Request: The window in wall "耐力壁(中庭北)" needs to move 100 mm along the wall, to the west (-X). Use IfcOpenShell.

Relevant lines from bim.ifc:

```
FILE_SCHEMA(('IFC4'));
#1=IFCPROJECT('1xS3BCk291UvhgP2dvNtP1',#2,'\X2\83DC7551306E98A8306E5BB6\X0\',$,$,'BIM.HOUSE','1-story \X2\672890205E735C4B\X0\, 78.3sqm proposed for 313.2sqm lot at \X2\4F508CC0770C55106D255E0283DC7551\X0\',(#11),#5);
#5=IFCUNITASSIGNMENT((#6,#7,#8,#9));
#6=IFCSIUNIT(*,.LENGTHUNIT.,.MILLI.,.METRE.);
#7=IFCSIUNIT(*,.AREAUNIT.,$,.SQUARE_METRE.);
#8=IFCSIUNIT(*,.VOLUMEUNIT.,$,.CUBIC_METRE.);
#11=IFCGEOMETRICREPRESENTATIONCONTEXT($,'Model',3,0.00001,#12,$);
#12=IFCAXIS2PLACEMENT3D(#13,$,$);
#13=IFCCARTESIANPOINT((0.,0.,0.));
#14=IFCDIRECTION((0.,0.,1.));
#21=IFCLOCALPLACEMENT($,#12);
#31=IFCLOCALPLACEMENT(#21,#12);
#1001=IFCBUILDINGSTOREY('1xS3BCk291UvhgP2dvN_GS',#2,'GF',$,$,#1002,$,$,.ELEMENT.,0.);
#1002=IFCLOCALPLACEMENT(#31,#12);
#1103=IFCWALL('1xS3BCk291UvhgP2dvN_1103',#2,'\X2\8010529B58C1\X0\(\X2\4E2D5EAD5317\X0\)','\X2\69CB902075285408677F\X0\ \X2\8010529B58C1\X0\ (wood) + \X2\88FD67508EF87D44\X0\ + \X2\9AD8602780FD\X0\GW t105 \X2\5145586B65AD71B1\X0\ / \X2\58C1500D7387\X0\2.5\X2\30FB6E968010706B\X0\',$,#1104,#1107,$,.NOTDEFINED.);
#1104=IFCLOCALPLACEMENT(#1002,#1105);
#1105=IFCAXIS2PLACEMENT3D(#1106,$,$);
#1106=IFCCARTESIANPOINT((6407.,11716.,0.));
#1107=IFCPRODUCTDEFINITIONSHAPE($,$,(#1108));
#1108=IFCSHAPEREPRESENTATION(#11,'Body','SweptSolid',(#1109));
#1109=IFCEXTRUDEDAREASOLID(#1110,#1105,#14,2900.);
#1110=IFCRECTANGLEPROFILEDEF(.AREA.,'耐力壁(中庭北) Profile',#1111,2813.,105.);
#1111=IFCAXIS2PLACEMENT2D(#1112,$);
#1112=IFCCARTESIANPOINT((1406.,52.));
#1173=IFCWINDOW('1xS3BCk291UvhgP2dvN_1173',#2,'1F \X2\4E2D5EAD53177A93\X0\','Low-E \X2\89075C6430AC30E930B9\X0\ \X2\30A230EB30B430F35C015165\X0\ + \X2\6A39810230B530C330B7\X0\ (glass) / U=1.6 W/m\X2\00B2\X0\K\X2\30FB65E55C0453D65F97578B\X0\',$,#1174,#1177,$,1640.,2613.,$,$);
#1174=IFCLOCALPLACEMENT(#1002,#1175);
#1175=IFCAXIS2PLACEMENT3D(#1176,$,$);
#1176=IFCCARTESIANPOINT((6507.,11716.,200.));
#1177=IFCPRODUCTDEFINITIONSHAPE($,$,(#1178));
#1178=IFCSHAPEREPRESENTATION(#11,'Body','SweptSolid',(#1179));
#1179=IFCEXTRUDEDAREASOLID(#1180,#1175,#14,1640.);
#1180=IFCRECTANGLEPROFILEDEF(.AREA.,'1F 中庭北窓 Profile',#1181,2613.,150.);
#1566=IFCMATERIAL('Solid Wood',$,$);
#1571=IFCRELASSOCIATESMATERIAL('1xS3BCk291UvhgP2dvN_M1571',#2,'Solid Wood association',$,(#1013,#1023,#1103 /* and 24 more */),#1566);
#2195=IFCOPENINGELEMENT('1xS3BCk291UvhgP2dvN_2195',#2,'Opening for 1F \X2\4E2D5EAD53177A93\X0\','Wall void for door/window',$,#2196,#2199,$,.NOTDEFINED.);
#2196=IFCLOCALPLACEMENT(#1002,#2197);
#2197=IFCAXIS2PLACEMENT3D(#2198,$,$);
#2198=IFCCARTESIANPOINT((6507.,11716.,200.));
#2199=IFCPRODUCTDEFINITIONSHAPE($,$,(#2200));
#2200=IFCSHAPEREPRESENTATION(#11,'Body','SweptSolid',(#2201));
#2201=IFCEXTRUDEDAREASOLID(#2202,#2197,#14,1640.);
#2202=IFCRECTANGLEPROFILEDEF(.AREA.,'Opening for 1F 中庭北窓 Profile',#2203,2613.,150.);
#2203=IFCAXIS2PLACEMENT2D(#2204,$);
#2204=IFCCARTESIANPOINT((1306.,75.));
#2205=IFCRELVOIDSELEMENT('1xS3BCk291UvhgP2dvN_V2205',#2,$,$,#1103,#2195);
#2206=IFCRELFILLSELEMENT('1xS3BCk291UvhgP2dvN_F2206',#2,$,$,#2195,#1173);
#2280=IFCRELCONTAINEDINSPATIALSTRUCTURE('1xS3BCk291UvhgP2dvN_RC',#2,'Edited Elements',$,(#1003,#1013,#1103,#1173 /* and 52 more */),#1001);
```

```python
import ifcopenshell
import ifcopenshell.api.geometry
import ifcopenshell.util.placement
import ifcopenshell.util.unit

model = ifcopenshell.open("bim.ifc")
unit_scale = ifcopenshell.util.unit.calculate_unit_scale(model)

window = model.by_guid("1xS3BCk291UvhgP2dvN_1173")
opening = window.FillsVoids[0].RelatingOpeningElement
wall = opening.VoidsElements[0].RelatingBuildingElement

wall_matrix = ifcopenshell.util.placement.get_local_placement(wall.ObjectPlacement)
shift = wall_matrix[:3, 0] * -0.1 / unit_scale
before = ifcopenshell.util.placement.get_local_placement(window.ObjectPlacement)[:3, 3].copy()

# The window is not placed relative to its opening, so move both.
for product in (opening, window):
    matrix = ifcopenshell.util.placement.get_local_placement(product.ObjectPlacement)
    matrix[:3, 3] += shift
    ifcopenshell.api.geometry.edit_object_placement(model, product=product, matrix=matrix, is_si=False)

after = ifcopenshell.util.placement.get_local_placement(window.ObjectPlacement)[:3, 3]
print("window moved by", (after - before).round(3) + 0.0)

model.write("bim_edited.ifc")
```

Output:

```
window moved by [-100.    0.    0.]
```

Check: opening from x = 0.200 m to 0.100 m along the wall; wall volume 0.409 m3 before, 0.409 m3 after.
